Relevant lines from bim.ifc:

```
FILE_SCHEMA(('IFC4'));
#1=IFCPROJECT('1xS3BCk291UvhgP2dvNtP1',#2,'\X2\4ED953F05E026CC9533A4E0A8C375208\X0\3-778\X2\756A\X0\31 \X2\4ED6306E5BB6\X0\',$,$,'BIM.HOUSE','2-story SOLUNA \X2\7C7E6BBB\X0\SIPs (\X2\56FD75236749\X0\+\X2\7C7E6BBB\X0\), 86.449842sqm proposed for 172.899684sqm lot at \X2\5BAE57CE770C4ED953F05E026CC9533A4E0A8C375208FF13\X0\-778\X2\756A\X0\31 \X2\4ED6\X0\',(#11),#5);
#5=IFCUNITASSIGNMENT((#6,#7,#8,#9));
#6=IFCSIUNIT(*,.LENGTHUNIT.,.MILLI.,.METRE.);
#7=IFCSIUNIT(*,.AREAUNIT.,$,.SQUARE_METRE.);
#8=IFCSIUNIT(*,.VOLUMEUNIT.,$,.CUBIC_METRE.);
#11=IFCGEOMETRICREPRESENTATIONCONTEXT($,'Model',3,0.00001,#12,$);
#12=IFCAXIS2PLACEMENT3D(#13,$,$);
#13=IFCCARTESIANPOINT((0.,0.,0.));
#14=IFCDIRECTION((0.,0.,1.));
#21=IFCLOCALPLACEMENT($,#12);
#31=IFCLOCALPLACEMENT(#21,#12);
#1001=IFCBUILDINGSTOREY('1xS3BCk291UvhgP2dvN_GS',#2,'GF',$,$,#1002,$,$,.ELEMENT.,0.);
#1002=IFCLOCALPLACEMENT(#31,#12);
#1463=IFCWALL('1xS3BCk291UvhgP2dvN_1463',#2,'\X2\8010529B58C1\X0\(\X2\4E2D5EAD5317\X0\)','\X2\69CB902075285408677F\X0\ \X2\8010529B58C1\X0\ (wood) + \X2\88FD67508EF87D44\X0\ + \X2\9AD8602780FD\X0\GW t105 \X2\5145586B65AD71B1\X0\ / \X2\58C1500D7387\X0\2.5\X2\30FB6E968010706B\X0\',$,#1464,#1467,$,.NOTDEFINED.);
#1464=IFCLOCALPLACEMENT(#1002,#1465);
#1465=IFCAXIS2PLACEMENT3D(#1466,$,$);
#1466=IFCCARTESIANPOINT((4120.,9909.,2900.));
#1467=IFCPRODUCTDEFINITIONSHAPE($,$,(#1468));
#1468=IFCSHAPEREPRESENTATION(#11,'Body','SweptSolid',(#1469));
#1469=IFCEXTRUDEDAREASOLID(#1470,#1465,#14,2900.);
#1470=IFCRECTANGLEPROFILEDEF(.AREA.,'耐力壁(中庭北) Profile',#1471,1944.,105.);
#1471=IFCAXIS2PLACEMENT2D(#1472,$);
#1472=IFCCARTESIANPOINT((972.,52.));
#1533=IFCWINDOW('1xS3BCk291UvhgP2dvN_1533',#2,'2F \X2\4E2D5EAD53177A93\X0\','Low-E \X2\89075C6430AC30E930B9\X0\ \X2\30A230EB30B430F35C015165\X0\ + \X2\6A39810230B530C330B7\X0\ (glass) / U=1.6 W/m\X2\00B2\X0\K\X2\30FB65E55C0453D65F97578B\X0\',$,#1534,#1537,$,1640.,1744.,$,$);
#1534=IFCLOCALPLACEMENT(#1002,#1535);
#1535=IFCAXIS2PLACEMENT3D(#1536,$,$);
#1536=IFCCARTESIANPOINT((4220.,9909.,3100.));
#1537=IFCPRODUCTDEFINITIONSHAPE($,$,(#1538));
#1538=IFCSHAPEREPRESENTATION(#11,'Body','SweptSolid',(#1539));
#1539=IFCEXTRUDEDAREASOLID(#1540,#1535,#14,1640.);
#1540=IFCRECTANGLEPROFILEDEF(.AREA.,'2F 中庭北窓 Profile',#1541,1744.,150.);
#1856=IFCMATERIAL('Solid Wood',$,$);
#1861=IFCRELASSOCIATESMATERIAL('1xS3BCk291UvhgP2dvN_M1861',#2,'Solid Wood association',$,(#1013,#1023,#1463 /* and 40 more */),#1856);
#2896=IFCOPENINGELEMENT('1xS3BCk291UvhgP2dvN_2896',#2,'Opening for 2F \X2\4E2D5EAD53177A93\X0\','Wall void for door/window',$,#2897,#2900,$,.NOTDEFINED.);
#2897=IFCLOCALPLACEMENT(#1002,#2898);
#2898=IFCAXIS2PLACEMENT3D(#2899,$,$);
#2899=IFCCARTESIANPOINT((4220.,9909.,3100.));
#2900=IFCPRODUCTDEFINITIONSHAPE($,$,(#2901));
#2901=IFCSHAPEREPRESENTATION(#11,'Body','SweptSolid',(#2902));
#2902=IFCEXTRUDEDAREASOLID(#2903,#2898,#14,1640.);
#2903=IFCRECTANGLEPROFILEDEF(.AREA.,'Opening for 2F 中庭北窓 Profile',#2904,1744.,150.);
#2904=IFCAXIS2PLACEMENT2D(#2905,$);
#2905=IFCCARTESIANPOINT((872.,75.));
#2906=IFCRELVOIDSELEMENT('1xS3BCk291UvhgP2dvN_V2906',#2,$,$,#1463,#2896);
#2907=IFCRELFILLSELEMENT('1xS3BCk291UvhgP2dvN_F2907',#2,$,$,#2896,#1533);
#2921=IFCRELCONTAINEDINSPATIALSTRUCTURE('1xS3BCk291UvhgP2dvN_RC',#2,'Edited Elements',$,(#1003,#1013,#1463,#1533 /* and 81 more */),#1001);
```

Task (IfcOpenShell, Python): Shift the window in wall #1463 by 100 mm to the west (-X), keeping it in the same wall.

```python
import ifcopenshell
import ifcopenshell.api.geometry
import ifcopenshell.util.placement

model = ifcopenshell.open("bim.ifc")

window = model.by_id(1533)
opening = window.FillsVoids[0].RelatingOpeningElement
wall = opening.VoidsElements[0].RelatingBuildingElement

wall_matrix = ifcopenshell.util.placement.get_local_placement(wall.ObjectPlacement)
shift = wall_matrix[:3, 0] * -100.0
before = ifcopenshell.util.placement.get_local_placement(window.ObjectPlacement)[:3, 3].copy()

# The window is not placed relative to its opening, so move both.
for product in (opening, window):
    matrix = ifcopenshell.util.placement.get_local_placement(product.ObjectPlacement)
    matrix[:3, 3] += shift
    ifcopenshell.api.geometry.edit_object_placement(model, product=product, matrix=matrix, is_si=False)

after = ifcopenshell.util.placement.get_local_placement(window.ObjectPlacement)[:3, 3]
print("window moved by", (after - before).round(3) + 0.0)

model.write("bim_edited.ifc")
```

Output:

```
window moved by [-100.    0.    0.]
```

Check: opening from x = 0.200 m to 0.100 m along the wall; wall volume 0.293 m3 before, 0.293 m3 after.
